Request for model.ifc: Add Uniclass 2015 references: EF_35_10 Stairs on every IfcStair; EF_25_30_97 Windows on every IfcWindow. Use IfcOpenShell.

First a look at what the model holds.

```python
import ifcopenshell

model = ifcopenshell.open("model.ifc")
print(model.schema)
print("classifications:", [c.Name for c in model.by_type("IfcClassification")])
for ifc_class in ("IfcDoor", "IfcRoof", "IfcStair", "IfcWall", "IfcWindow"):
    print(ifc_class, len(model.by_type(ifc_class)))
```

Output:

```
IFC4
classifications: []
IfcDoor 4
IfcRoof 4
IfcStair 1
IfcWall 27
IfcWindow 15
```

```python
import ifcopenshell
import ifcopenshell.api.classification

model = ifcopenshell.open("model.ifc")

system = ifcopenshell.api.classification.add_classification(model, classification="Uniclass 2015")

codes = {
    "IfcStair": ("EF_35_10", "Stairs"),
    "IfcWindow": ("EF_25_30_97", "Windows"),
}
for ifc_class, (code, name) in codes.items():
    products = model.by_type(ifc_class)
    ifcopenshell.api.classification.add_reference(
        model, products=products, classification=system, identification=code, name=name
    )
    print(code, len(products))

model.write("model_rev.ifc")
```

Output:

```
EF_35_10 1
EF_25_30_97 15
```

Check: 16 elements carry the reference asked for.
